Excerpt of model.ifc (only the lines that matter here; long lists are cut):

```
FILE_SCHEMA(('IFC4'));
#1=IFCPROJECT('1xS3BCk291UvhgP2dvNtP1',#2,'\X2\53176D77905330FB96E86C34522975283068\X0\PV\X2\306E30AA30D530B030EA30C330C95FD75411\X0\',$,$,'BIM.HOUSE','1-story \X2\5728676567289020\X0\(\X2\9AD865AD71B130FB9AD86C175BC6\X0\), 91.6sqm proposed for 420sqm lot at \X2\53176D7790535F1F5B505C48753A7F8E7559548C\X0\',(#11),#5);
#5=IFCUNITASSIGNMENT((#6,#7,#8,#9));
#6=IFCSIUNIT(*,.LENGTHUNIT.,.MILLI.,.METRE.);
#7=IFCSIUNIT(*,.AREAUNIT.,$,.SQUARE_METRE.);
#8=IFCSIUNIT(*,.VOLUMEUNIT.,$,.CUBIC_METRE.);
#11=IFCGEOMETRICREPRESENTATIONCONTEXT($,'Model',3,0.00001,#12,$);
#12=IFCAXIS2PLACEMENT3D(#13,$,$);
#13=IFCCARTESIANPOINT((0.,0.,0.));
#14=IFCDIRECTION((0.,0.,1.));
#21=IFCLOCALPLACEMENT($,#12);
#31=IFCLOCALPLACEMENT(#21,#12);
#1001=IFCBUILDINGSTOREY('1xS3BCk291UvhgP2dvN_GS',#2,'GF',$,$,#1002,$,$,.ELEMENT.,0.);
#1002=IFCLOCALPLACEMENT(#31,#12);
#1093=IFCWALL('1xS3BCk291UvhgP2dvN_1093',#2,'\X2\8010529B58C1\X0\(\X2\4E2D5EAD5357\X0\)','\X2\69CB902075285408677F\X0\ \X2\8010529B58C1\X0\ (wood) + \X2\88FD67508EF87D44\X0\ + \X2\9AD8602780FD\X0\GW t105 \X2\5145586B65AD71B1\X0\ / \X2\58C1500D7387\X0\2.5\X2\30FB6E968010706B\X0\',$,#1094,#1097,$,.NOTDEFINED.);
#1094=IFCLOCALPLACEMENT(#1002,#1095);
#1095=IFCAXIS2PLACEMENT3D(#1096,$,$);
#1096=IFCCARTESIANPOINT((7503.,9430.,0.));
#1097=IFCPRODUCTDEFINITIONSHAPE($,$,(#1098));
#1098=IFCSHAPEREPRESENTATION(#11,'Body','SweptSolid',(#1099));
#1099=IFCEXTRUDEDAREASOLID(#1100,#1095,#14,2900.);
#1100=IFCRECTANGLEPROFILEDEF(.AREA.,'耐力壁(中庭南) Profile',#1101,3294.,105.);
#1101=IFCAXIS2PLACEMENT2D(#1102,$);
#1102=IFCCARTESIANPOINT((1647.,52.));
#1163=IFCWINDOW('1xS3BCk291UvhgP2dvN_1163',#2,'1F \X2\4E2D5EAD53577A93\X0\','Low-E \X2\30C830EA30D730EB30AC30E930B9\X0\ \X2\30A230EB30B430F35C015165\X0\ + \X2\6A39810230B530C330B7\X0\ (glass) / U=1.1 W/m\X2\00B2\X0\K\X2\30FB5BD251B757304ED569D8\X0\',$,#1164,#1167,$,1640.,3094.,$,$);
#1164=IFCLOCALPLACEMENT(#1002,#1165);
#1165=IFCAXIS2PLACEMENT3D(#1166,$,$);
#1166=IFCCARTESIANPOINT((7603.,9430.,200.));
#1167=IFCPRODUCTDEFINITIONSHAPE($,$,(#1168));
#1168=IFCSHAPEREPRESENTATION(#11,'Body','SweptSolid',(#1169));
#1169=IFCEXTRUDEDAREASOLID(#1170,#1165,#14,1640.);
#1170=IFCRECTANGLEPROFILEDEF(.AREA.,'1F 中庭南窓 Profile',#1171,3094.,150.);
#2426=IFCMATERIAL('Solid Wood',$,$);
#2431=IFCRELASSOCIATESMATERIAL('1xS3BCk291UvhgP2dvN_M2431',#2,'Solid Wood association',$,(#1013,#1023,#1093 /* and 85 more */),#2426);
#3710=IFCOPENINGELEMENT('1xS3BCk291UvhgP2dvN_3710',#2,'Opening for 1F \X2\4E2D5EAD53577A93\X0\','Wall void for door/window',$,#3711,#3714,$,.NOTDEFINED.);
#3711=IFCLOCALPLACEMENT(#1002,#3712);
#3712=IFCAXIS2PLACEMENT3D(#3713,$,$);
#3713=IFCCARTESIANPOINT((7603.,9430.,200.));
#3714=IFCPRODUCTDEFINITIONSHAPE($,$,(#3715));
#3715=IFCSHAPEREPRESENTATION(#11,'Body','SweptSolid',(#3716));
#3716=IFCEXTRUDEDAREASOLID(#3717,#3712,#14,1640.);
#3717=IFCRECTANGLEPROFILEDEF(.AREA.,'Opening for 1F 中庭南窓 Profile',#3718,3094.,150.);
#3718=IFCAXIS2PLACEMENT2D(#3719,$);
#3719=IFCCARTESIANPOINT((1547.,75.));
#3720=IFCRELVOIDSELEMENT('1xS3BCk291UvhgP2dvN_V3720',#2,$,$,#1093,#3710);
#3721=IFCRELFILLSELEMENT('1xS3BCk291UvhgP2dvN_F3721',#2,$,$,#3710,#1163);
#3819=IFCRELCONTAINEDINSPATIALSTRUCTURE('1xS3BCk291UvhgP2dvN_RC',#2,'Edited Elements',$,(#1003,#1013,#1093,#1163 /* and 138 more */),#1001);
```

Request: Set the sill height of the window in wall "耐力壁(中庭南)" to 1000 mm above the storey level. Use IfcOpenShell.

```python
import numpy as np
import ifcopenshell
import ifcopenshell.api.geometry
import ifcopenshell.geom
import ifcopenshell.util.element
import ifcopenshell.util.placement
import ifcopenshell.util.shape
import ifcopenshell.util.unit

model = ifcopenshell.open("model.ifc")
unit_scale = ifcopenshell.util.unit.calculate_unit_scale(model)

window = model.by_guid("1xS3BCk291UvhgP2dvN_1163")
opening = window.FillsVoids[0].RelatingOpeningElement
storey = ifcopenshell.util.element.get_container(window, ifc_class="IfcBuildingStorey")
level = ifcopenshell.util.placement.get_local_placement(storey.ObjectPlacement)[2, 3]

# The opening's origin need not be at the sill, so measure its lowest point.
shape = ifcopenshell.geom.create_shape(ifcopenshell.geom.settings(), opening)
bottom = ifcopenshell.util.shape.get_shape_bottom_elevation(shape, shape.geometry) / unit_scale
dz = level + 1 / unit_scale - bottom

shift = np.array([0.0, 0.0, dz])
# The window is not placed relative to its opening, so move both.
for product in (opening, window):
    matrix = ifcopenshell.util.placement.get_local_placement(product.ObjectPlacement)
    matrix[:3, 3] += shift
    ifcopenshell.api.geometry.edit_object_placement(model, product=product, matrix=matrix, is_si=False)

print(f"moved by {dz * unit_scale:+.3f} m")

model.write("model_edited.ifc")
```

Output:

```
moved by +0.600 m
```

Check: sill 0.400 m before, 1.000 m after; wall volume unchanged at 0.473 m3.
